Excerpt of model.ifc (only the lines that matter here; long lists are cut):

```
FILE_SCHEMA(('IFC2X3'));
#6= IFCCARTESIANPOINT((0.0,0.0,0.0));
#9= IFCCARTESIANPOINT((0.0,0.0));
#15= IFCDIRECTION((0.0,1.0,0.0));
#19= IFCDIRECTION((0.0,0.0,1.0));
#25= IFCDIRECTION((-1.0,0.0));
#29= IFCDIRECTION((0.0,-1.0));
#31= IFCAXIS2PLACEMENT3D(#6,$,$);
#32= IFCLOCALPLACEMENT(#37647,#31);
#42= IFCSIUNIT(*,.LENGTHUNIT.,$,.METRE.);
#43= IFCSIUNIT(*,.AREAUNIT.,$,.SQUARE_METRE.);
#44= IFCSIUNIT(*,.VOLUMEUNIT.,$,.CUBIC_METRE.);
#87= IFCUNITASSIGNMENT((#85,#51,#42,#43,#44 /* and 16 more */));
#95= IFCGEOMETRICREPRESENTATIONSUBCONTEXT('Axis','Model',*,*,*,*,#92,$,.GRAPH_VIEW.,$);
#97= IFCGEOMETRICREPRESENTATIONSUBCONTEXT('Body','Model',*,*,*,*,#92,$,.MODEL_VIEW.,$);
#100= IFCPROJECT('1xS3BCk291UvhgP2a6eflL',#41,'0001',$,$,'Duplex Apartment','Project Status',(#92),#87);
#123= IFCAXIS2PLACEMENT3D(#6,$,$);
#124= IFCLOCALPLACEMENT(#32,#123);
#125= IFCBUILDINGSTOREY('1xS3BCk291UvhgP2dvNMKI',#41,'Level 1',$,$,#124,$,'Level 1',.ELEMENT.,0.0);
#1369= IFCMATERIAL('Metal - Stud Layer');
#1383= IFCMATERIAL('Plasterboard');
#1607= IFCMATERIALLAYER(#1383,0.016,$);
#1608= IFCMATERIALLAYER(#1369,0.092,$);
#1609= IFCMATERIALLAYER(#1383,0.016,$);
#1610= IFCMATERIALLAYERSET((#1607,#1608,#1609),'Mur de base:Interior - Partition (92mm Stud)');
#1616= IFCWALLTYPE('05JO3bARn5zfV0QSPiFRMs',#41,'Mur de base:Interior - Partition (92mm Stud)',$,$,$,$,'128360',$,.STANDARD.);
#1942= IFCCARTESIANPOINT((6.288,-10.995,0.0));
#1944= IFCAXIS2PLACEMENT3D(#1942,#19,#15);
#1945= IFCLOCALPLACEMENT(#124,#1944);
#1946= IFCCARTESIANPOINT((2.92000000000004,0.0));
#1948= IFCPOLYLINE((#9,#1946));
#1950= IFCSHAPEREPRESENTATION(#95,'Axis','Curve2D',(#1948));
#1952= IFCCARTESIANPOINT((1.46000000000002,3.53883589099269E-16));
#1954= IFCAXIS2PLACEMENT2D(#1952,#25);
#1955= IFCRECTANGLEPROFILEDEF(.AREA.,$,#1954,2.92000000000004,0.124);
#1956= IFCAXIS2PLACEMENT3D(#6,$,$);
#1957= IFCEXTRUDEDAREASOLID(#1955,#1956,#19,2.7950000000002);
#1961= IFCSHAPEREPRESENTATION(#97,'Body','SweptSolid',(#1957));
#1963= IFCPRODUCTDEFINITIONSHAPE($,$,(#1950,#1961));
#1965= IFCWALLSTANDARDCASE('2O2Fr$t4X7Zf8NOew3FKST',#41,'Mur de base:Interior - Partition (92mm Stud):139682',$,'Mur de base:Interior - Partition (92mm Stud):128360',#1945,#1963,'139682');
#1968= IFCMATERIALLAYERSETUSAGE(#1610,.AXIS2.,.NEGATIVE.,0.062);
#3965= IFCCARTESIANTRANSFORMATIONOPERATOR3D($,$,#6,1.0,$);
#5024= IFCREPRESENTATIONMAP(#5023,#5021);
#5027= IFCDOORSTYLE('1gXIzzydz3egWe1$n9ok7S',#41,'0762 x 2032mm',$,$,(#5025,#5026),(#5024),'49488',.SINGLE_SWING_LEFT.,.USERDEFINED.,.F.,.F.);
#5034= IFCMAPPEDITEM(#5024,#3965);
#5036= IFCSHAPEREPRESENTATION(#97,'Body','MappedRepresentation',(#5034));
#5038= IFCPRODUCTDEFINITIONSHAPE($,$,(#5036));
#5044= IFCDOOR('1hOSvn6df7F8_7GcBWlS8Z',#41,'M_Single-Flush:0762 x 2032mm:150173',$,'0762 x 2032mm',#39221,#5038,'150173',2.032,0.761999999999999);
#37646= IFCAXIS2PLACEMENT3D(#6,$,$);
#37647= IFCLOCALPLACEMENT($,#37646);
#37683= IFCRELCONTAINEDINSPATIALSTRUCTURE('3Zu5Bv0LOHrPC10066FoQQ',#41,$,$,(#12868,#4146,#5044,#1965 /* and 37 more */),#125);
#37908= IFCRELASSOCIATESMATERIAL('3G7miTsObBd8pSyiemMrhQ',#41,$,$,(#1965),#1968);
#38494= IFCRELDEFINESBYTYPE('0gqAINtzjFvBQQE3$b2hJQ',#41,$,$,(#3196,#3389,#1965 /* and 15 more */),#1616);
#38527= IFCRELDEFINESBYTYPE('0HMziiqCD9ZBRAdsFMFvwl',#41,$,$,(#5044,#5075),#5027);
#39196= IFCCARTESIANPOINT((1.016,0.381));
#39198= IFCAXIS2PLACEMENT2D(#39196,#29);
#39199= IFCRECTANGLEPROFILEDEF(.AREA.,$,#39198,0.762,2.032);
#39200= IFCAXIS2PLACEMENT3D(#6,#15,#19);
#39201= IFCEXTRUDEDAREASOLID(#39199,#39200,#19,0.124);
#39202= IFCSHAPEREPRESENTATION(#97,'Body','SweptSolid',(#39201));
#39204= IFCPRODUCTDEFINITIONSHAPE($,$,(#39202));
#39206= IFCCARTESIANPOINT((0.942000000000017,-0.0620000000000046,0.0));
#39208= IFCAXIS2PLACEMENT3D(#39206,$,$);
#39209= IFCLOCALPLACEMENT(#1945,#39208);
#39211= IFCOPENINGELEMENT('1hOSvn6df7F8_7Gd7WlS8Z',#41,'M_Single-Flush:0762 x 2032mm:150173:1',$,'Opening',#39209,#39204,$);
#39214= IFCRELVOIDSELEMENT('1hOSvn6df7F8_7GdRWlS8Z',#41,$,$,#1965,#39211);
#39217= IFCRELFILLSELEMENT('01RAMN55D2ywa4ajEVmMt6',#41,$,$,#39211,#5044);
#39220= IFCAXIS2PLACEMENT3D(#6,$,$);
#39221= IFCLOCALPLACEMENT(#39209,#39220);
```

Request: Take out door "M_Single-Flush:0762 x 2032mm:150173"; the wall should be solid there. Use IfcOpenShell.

```python
import ifcopenshell
import ifcopenshell.api.feature
import ifcopenshell.api.root
import ifcopenshell.geom
import ifcopenshell.util.shape

model = ifcopenshell.open("model.ifc")
settings = ifcopenshell.geom.settings()


def volume(element):
    """Net volume in cubic metres, openings subtracted."""
    shape = ifcopenshell.geom.create_shape(settings, element)
    return ifcopenshell.util.shape.get_volume(shape.geometry)


door = model.by_guid("1hOSvn6df7F8_7GcBWlS8Z")
opening = door.FillsVoids[0].RelatingOpeningElement
wall = opening.VoidsElements[0].RelatingBuildingElement
before = volume(wall)

ifcopenshell.api.root.remove_product(model, product=door)
ifcopenshell.api.feature.remove_feature(model, feature=opening)

after = volume(wall)

print(f"wall volume {before:.3f} -> {after:.3f} m3")

model.write("model_v2.ifc")
```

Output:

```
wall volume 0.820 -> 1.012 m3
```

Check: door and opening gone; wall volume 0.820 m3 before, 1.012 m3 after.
